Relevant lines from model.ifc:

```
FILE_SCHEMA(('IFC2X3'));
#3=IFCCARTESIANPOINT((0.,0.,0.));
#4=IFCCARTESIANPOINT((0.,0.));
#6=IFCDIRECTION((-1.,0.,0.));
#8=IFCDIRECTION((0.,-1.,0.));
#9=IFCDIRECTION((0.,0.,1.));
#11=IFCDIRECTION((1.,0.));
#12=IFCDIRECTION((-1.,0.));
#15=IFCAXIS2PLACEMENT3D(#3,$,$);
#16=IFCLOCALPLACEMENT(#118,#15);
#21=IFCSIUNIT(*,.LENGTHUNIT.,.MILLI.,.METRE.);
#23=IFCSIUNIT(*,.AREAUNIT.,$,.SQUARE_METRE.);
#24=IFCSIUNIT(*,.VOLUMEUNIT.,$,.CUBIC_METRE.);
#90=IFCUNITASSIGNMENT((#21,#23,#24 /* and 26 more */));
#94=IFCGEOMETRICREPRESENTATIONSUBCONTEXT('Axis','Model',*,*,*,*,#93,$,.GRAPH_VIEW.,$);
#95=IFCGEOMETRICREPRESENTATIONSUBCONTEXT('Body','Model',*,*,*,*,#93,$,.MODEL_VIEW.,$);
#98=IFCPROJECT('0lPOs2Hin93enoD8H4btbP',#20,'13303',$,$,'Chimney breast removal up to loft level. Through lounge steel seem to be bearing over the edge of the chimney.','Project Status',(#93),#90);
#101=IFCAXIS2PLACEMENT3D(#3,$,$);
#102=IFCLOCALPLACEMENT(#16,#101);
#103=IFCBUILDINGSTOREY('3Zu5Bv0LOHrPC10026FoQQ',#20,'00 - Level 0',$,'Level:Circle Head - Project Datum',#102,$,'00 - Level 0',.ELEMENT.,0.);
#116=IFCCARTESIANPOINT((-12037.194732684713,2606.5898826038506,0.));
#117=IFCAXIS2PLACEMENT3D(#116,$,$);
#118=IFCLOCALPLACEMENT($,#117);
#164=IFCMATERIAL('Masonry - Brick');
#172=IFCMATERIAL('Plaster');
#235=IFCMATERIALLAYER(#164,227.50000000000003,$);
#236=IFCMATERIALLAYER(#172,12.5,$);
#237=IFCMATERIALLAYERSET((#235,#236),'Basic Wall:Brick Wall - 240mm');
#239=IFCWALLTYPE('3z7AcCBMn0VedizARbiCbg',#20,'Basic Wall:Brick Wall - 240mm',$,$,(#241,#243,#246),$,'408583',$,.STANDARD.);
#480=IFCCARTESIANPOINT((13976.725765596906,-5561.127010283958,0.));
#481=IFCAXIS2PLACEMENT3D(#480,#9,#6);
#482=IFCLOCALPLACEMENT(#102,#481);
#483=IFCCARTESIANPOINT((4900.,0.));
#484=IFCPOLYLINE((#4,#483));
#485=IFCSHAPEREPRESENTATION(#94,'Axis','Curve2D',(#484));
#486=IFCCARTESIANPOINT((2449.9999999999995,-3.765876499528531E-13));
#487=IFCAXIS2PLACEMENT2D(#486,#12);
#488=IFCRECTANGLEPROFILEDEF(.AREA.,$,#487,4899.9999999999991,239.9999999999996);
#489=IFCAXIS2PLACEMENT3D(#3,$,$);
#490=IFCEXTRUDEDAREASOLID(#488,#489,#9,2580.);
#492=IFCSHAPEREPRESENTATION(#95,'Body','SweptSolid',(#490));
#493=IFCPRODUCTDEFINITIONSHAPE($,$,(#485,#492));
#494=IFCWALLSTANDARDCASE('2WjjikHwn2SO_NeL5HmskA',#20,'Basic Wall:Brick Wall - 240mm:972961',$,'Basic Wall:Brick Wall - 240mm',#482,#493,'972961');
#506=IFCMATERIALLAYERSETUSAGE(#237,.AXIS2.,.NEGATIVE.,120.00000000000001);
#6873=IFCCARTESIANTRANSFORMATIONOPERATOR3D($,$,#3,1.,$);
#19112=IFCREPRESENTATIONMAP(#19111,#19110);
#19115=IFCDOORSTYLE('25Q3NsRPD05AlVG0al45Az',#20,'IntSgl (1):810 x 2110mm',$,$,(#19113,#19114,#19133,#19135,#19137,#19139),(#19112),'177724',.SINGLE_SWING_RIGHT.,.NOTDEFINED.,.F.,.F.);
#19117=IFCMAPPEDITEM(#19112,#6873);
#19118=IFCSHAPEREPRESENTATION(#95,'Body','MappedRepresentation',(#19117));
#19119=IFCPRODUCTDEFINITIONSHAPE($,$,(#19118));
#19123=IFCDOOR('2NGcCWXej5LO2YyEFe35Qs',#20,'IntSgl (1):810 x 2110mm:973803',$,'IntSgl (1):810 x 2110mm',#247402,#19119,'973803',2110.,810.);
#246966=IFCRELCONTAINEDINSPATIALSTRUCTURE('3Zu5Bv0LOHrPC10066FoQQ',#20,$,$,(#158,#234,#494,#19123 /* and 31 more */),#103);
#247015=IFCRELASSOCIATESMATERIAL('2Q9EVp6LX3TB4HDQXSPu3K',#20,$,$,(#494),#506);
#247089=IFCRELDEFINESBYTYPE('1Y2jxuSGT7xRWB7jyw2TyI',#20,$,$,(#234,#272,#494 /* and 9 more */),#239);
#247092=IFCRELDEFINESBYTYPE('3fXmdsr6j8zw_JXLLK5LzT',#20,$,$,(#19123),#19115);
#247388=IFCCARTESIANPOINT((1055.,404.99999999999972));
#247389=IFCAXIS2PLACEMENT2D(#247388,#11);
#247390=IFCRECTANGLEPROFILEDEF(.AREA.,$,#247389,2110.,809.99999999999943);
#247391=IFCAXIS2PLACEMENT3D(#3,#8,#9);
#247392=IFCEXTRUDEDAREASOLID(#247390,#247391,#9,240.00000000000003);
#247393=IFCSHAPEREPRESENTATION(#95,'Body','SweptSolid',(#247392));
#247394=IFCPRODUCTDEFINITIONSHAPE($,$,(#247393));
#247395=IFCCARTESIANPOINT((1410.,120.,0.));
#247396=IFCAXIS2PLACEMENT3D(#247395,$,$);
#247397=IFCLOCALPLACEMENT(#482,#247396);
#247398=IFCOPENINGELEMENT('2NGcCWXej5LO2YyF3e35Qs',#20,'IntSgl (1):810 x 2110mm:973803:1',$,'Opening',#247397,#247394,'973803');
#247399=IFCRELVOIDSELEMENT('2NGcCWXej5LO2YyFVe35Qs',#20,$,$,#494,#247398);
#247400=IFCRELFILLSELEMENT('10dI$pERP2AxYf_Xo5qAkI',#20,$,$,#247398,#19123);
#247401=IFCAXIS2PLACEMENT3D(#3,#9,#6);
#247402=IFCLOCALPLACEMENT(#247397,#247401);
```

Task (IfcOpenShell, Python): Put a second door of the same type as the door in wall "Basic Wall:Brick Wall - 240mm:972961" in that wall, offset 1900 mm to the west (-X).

```python
import ifcopenshell
import ifcopenshell.api.feature
import ifcopenshell.api.geometry
import ifcopenshell.api.root
import ifcopenshell.geom
import ifcopenshell.util.element
import ifcopenshell.util.placement
import ifcopenshell.util.shape

model = ifcopenshell.open("model.ifc")
settings = ifcopenshell.geom.settings()


def volume(element):
    """Net volume in cubic metres, openings subtracted."""
    shape = ifcopenshell.geom.create_shape(settings, element)
    return ifcopenshell.util.shape.get_volume(shape.geometry)


def reuse_history(source, copy):
    """copy_class also copies each property set's owner history, people and application; keep the originals."""
    for rel in copy.IsDefinedBy:
        if rel.is_a("IfcRelDefinesByProperties") and (history := rel.RelatingPropertyDefinition.OwnerHistory):
            rel.RelatingPropertyDefinition.OwnerHistory = source.OwnerHistory
            ifcopenshell.util.element.remove_deep2(model, history)


door = model.by_guid("2NGcCWXej5LO2YyEFe35Qs")
opening = door.FillsVoids[0].RelatingOpeningElement
wall = opening.VoidsElements[0].RelatingBuildingElement
before = volume(wall)
shift = ifcopenshell.util.placement.get_local_placement(wall.ObjectPlacement)[:3, 0] * 1900.0

# copy_class copies the void relationship, type, container and properties, but no geometry.
new_opening = ifcopenshell.api.root.copy_class(model, product=opening)
new_opening.Representation = ifcopenshell.util.element.copy_deep(
    model, opening.Representation, exclude=["IfcGeometricRepresentationContext", "IfcRepresentationMap"]
)
new_opening.Name = "IntSgl (1):810 x 2110mm"
new_opening.Tag = None
new_door = ifcopenshell.api.root.copy_class(model, product=door)
new_door.Representation = ifcopenshell.util.element.copy_deep(
    model, door.Representation, exclude=["IfcGeometricRepresentationContext", "IfcRepresentationMap"]
)
new_door.Name = "IntSgl (1):810 x 2110mm"
new_door.Tag = None
reuse_history(door, new_door)
fills = ifcopenshell.api.feature.add_filling(model, opening=new_opening, element=new_door)
fills.OwnerHistory = new_door.OwnerHistory  # required in IFC2X3

for old, new in ((opening, new_opening), (door, new_door)):
    matrix = ifcopenshell.util.placement.get_local_placement(old.ObjectPlacement)
    matrix[:3, 3] += shift
    ifcopenshell.api.geometry.edit_object_placement(model, product=new, matrix=matrix, is_si=False)

after = volume(wall)

print(f"wall volume {before:.3f} -> {after:.3f} m3")

model.write("model_updated.ifc")
```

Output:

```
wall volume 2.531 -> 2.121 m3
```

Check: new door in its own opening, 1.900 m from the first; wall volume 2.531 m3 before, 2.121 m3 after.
